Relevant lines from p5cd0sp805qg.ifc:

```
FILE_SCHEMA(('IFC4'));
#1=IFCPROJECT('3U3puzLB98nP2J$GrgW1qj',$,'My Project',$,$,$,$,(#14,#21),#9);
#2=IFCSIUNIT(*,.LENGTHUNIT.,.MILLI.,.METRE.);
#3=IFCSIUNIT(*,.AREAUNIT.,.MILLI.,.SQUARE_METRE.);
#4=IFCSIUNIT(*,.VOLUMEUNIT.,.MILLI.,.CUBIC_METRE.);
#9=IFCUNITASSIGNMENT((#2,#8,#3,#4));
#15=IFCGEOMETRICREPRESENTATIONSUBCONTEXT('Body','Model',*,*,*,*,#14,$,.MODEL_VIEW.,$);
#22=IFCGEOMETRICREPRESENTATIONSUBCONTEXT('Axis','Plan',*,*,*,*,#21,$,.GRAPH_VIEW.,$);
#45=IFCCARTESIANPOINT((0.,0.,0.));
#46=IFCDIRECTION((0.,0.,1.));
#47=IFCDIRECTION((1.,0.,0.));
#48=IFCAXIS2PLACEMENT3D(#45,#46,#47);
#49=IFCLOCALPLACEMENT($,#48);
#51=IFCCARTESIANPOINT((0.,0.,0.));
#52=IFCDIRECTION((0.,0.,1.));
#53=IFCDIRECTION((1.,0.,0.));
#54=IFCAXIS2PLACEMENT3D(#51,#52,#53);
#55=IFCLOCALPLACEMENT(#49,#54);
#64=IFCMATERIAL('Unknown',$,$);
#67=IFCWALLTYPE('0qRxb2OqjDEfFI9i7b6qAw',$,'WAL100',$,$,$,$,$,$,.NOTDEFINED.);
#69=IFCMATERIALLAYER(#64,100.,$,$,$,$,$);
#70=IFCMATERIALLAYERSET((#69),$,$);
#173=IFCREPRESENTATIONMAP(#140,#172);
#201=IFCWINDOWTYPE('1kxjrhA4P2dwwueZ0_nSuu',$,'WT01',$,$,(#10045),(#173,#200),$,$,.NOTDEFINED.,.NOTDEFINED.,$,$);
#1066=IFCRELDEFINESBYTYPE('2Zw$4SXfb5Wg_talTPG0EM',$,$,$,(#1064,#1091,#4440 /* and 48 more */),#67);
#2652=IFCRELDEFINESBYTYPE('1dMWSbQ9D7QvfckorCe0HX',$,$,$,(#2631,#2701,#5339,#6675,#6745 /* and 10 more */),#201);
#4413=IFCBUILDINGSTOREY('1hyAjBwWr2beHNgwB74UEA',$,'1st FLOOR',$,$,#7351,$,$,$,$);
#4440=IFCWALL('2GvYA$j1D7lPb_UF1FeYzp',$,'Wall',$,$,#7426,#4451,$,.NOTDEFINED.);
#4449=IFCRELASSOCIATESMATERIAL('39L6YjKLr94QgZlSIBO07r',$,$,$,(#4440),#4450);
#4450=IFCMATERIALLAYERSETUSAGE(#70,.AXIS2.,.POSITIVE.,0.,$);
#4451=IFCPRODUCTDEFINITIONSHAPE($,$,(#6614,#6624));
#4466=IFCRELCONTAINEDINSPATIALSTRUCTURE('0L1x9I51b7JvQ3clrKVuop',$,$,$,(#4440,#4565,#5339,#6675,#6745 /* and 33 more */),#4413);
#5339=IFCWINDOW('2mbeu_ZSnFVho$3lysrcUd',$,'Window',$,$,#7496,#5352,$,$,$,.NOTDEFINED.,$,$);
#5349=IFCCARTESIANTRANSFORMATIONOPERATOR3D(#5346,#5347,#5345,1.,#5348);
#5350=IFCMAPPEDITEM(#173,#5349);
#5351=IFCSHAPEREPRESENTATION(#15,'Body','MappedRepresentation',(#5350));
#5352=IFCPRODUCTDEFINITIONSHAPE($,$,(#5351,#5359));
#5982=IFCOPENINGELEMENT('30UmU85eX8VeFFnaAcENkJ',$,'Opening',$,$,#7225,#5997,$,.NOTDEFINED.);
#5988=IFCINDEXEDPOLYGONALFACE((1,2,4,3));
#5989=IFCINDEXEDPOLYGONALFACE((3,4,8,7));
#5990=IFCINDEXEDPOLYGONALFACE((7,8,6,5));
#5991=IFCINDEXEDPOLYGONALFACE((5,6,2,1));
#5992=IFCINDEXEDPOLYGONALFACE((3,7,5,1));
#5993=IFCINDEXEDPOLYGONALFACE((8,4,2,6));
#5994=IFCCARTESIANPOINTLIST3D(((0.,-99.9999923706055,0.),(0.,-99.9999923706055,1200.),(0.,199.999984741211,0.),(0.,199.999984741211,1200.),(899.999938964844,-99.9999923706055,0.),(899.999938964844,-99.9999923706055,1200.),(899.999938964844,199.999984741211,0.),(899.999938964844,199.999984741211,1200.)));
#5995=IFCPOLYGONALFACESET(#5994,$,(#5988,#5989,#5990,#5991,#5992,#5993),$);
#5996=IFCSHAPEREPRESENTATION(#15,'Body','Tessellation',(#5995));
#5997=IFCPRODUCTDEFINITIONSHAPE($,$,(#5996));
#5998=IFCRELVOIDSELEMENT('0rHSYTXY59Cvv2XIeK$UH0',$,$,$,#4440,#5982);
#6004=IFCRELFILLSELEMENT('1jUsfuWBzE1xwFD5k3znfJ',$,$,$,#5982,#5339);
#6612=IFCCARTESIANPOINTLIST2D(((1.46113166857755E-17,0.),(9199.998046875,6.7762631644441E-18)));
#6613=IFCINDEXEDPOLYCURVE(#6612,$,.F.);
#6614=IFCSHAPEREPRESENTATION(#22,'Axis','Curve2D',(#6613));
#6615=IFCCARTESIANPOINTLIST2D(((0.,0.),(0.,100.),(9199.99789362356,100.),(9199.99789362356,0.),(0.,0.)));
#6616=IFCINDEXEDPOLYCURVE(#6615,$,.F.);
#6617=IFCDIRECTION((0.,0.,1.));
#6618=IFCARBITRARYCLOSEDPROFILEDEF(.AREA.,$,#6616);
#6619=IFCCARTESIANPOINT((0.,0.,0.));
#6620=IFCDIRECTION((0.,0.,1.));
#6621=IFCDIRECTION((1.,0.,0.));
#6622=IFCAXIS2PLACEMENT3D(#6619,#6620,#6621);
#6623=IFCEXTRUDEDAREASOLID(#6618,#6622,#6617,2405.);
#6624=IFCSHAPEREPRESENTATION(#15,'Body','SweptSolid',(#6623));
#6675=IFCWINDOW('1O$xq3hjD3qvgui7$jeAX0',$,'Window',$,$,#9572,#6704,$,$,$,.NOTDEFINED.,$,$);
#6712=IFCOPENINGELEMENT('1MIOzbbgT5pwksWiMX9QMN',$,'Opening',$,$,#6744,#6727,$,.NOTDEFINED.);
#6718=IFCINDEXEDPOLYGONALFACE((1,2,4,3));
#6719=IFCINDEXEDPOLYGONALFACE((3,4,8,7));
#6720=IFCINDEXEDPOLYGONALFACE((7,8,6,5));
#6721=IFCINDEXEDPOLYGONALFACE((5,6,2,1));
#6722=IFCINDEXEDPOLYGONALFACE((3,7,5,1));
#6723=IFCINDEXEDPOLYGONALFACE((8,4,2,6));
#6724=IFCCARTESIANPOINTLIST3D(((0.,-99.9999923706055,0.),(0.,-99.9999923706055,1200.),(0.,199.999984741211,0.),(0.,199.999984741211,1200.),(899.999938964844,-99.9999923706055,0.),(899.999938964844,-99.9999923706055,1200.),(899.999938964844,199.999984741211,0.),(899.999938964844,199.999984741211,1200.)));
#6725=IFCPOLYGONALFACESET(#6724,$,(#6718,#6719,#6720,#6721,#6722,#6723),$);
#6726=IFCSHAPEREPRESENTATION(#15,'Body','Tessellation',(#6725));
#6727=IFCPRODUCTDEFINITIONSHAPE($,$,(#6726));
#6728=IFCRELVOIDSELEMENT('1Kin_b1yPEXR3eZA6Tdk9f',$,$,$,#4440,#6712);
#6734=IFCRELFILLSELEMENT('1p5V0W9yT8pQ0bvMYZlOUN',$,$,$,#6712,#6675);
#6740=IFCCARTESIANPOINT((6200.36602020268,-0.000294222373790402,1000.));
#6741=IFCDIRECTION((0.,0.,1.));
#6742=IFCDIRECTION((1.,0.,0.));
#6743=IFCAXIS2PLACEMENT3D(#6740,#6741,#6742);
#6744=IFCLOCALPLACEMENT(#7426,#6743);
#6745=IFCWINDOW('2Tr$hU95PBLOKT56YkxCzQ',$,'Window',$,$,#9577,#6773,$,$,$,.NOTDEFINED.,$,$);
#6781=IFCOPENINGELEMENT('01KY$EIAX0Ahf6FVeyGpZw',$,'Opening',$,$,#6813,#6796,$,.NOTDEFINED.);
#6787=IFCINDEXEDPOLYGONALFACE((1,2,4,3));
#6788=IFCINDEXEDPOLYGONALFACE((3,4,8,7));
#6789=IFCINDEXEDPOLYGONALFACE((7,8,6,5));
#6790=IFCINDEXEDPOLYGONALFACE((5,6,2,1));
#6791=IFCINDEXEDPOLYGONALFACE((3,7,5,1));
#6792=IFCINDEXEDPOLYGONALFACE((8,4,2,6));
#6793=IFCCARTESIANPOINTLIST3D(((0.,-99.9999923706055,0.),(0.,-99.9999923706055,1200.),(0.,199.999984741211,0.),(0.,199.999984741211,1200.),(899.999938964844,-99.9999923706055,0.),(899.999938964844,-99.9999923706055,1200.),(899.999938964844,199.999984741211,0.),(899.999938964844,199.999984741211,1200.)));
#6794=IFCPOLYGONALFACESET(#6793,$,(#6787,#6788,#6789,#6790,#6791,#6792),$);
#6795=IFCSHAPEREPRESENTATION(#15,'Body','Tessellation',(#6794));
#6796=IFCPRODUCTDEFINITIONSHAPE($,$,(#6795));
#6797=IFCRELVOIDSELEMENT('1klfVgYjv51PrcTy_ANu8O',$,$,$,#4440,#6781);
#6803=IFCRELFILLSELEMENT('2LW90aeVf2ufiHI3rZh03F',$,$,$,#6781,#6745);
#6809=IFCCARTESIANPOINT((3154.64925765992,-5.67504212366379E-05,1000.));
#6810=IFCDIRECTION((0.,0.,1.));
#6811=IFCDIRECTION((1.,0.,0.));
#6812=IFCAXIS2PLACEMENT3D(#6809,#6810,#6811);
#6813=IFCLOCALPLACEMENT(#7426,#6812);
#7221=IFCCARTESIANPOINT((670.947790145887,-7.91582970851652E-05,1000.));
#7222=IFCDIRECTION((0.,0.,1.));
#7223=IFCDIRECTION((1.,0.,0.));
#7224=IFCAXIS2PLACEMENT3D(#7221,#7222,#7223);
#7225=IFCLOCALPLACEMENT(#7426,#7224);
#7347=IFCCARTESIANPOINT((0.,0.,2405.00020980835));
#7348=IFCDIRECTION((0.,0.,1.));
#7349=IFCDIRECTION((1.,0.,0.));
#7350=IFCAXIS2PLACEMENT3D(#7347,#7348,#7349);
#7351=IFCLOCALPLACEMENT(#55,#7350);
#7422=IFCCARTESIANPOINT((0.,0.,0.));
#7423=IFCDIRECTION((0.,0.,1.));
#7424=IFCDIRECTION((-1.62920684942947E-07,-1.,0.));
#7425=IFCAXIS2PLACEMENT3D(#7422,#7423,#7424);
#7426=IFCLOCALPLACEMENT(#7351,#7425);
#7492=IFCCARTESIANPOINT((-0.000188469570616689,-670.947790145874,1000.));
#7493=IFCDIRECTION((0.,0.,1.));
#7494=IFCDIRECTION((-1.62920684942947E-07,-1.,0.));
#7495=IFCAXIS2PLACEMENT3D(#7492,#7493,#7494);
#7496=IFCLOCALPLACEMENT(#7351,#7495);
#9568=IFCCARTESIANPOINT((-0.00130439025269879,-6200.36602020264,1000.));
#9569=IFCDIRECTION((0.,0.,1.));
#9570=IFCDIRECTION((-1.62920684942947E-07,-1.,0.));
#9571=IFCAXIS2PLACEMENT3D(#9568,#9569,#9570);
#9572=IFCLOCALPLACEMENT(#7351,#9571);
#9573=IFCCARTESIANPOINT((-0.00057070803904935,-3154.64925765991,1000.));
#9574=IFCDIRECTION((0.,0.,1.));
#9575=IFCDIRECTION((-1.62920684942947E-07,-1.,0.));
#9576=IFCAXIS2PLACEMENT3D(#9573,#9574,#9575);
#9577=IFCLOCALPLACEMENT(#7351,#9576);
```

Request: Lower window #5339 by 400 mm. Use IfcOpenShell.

```python
import numpy as np
import ifcopenshell
import ifcopenshell.api.geometry
import ifcopenshell.util.placement
import ifcopenshell.util.unit

model = ifcopenshell.open("p5cd0sp805qg.ifc")
unit_scale = ifcopenshell.util.unit.calculate_unit_scale(model)

window = model.by_id(5339)
opening = window.FillsVoids[0].RelatingOpeningElement
dz = -400.0

shift = np.array([0.0, 0.0, dz])
# The window is not placed relative to its opening, so move both.
for product in (opening, window):
    matrix = ifcopenshell.util.placement.get_local_placement(product.ObjectPlacement)
    matrix[:3, 3] += shift
    ifcopenshell.api.geometry.edit_object_placement(model, product=product, matrix=matrix, is_si=False)

print(f"moved by {dz * unit_scale:+.3f} m")

model.write("p5cd0sp805qg_edited.ifc")
```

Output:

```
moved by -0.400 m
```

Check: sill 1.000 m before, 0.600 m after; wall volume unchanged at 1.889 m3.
